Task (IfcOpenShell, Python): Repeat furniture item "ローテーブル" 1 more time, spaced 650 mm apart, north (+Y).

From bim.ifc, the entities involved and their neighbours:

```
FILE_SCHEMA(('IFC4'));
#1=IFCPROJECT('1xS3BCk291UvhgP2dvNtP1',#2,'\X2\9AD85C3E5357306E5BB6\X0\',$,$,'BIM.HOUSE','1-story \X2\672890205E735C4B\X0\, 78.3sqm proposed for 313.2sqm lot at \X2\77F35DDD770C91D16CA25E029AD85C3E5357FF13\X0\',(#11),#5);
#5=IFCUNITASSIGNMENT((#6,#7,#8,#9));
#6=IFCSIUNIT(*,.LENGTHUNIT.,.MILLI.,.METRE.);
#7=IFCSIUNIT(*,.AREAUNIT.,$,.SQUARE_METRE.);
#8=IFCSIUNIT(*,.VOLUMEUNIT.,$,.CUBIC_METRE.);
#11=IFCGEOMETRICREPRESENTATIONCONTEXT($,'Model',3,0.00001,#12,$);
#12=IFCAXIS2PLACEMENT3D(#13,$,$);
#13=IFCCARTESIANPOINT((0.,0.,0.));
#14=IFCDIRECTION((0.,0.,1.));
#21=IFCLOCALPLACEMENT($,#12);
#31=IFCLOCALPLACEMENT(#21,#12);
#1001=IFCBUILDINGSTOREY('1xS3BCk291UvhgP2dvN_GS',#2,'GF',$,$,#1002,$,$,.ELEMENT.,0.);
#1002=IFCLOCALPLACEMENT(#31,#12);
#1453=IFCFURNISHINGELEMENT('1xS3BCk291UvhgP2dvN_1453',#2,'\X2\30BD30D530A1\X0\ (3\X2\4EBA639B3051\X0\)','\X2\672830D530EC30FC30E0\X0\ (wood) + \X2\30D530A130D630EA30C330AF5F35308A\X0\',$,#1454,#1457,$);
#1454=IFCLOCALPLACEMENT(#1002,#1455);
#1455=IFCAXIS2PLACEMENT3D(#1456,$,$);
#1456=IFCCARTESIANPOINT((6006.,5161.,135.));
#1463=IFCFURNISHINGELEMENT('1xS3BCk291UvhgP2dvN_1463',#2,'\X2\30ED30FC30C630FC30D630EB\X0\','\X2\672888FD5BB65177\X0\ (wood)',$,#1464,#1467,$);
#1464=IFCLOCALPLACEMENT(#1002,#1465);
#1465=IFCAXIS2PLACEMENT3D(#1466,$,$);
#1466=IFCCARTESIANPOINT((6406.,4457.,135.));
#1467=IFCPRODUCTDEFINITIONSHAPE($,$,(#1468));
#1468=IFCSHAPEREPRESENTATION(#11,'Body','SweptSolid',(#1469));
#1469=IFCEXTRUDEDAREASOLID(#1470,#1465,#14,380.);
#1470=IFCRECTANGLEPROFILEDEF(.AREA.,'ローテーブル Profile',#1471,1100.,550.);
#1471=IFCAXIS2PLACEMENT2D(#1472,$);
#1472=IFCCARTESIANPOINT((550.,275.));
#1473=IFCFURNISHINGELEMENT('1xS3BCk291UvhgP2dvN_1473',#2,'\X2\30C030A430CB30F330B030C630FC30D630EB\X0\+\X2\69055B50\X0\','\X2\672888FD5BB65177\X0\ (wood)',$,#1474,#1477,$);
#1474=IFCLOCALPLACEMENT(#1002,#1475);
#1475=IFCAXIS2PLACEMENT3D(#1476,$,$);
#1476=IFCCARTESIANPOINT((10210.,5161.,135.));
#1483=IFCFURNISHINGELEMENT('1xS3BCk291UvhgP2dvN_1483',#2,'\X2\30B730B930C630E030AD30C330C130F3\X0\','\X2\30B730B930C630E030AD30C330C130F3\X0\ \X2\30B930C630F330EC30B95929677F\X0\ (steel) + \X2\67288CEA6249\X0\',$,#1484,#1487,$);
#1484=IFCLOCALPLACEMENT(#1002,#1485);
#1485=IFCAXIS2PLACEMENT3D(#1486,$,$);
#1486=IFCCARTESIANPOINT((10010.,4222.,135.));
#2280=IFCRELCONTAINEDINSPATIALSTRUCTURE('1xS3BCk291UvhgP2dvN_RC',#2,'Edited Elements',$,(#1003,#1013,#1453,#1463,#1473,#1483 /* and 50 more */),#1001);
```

```python
import numpy as np
import ifcopenshell
import ifcopenshell.api.geometry
import ifcopenshell.api.root
import ifcopenshell.util.element
import ifcopenshell.util.placement
import ifcopenshell.util.unit

model = ifcopenshell.open("bim.ifc")
unit_scale = ifcopenshell.util.unit.calculate_unit_scale(model)


def reuse_history(source, copy):
    """copy_class also copies each property set's owner history, people and application; keep the originals."""
    for rel in copy.IsDefinedBy:
        if rel.is_a("IfcRelDefinesByProperties") and (history := rel.RelatingPropertyDefinition.OwnerHistory):
            rel.RelatingPropertyDefinition.OwnerHistory = source.OwnerHistory
            ifcopenshell.util.element.remove_deep2(model, history)


source = model.by_id(1463)
base = ifcopenshell.util.placement.get_local_placement(source.ObjectPlacement)
step = np.array([0.0, 1.0, 0.0]) * 0.65 / unit_scale

for i in range(1, 2):
    copy = ifcopenshell.api.root.copy_class(model, product=source)
    copy.Representation = ifcopenshell.util.element.copy_deep(
        model, source.Representation, exclude=["IfcGeometricRepresentationContext", "IfcRepresentationMap"]
    )
    reuse_history(source, copy)
    matrix = base.copy()
    matrix[:3, 3] += i * step
    print("added at", matrix[:3, 3].round(3) + 0.0)
    ifcopenshell.api.geometry.edit_object_placement(model, product=copy, matrix=matrix, is_si=False)

model.write("bim_v2.ifc")
```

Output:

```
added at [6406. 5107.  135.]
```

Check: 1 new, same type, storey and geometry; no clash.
